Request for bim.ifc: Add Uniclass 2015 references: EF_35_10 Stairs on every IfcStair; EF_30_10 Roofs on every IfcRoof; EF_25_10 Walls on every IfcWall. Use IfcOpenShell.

First a look at what the model holds.

```python
import ifcopenshell

model = ifcopenshell.open("bim.ifc")
print(model.schema)
print("classifications:", [c.Name for c in model.by_type("IfcClassification")])
for ifc_class in ("IfcDoor", "IfcRoof", "IfcStair", "IfcWall", "IfcWindow"):
    print(ifc_class, len(model.by_type(ifc_class)))
```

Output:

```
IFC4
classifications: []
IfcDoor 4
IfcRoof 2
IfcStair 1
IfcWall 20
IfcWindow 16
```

```python
import ifcopenshell
import ifcopenshell.api.classification

model = ifcopenshell.open("bim.ifc")

system = ifcopenshell.api.classification.add_classification(model, classification="Uniclass 2015")

codes = {
    "IfcStair": ("EF_35_10", "Stairs"),
    "IfcRoof": ("EF_30_10", "Roofs"),
    "IfcWall": ("EF_25_10", "Walls"),
}
for ifc_class, (code, name) in codes.items():
    products = model.by_type(ifc_class)
    ifcopenshell.api.classification.add_reference(
        model, products=products, classification=system, identification=code, name=name
    )
    print(code, len(products))

model.write("bim_edited.ifc")
```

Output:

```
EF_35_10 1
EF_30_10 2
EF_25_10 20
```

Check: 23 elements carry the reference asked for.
